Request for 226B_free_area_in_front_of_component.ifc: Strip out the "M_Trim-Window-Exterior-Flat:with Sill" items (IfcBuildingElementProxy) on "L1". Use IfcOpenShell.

First a look at what the model holds.

```python
import ifcopenshell
import ifcopenshell.util.element

model = ifcopenshell.open("226B_free_area_in_front_of_component.ifc")
print(model.schema)
storey = next(s for s in model.by_type("IfcBuildingStorey") if s.Name == "L1")
proxies = [e for e in ifcopenshell.util.element.get_decomposition(storey) if e.is_a("IfcBuildingElementProxy")]
seen = {}
for e in proxies:
    element_type = ifcopenshell.util.element.get_type(e)
    name = element_type.Name if element_type not in (None, e) else None
    seen[name] = seen.get(name, 0) + 1
for name, count in sorted(seen.items(), key=str):
    print(count, "x", name)
```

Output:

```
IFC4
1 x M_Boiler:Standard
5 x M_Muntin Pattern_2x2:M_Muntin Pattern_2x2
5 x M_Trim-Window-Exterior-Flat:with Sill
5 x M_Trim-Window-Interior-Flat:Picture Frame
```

```python
import ifcopenshell
import ifcopenshell.api.root
import ifcopenshell.util.element

model = ifcopenshell.open("226B_free_area_in_front_of_component.ifc")

storey = next(s for s in model.by_type("IfcBuildingStorey") if s.Name == "L1")
proxies = [e for e in ifcopenshell.util.element.get_decomposition(storey) if e.is_a("IfcBuildingElementProxy")]
targets = [e for e in proxies if (t := ifcopenshell.util.element.get_type(e)) not in (None, e) and t.Name == "M_Trim-Window-Exterior-Flat:with Sill"]

for e in targets:
    ifcopenshell.api.root.remove_product(model, product=e)
print(len(targets), "removed")

model.write("226B_free_area_in_front_of_component_rev.ifc")
```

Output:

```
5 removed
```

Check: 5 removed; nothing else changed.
